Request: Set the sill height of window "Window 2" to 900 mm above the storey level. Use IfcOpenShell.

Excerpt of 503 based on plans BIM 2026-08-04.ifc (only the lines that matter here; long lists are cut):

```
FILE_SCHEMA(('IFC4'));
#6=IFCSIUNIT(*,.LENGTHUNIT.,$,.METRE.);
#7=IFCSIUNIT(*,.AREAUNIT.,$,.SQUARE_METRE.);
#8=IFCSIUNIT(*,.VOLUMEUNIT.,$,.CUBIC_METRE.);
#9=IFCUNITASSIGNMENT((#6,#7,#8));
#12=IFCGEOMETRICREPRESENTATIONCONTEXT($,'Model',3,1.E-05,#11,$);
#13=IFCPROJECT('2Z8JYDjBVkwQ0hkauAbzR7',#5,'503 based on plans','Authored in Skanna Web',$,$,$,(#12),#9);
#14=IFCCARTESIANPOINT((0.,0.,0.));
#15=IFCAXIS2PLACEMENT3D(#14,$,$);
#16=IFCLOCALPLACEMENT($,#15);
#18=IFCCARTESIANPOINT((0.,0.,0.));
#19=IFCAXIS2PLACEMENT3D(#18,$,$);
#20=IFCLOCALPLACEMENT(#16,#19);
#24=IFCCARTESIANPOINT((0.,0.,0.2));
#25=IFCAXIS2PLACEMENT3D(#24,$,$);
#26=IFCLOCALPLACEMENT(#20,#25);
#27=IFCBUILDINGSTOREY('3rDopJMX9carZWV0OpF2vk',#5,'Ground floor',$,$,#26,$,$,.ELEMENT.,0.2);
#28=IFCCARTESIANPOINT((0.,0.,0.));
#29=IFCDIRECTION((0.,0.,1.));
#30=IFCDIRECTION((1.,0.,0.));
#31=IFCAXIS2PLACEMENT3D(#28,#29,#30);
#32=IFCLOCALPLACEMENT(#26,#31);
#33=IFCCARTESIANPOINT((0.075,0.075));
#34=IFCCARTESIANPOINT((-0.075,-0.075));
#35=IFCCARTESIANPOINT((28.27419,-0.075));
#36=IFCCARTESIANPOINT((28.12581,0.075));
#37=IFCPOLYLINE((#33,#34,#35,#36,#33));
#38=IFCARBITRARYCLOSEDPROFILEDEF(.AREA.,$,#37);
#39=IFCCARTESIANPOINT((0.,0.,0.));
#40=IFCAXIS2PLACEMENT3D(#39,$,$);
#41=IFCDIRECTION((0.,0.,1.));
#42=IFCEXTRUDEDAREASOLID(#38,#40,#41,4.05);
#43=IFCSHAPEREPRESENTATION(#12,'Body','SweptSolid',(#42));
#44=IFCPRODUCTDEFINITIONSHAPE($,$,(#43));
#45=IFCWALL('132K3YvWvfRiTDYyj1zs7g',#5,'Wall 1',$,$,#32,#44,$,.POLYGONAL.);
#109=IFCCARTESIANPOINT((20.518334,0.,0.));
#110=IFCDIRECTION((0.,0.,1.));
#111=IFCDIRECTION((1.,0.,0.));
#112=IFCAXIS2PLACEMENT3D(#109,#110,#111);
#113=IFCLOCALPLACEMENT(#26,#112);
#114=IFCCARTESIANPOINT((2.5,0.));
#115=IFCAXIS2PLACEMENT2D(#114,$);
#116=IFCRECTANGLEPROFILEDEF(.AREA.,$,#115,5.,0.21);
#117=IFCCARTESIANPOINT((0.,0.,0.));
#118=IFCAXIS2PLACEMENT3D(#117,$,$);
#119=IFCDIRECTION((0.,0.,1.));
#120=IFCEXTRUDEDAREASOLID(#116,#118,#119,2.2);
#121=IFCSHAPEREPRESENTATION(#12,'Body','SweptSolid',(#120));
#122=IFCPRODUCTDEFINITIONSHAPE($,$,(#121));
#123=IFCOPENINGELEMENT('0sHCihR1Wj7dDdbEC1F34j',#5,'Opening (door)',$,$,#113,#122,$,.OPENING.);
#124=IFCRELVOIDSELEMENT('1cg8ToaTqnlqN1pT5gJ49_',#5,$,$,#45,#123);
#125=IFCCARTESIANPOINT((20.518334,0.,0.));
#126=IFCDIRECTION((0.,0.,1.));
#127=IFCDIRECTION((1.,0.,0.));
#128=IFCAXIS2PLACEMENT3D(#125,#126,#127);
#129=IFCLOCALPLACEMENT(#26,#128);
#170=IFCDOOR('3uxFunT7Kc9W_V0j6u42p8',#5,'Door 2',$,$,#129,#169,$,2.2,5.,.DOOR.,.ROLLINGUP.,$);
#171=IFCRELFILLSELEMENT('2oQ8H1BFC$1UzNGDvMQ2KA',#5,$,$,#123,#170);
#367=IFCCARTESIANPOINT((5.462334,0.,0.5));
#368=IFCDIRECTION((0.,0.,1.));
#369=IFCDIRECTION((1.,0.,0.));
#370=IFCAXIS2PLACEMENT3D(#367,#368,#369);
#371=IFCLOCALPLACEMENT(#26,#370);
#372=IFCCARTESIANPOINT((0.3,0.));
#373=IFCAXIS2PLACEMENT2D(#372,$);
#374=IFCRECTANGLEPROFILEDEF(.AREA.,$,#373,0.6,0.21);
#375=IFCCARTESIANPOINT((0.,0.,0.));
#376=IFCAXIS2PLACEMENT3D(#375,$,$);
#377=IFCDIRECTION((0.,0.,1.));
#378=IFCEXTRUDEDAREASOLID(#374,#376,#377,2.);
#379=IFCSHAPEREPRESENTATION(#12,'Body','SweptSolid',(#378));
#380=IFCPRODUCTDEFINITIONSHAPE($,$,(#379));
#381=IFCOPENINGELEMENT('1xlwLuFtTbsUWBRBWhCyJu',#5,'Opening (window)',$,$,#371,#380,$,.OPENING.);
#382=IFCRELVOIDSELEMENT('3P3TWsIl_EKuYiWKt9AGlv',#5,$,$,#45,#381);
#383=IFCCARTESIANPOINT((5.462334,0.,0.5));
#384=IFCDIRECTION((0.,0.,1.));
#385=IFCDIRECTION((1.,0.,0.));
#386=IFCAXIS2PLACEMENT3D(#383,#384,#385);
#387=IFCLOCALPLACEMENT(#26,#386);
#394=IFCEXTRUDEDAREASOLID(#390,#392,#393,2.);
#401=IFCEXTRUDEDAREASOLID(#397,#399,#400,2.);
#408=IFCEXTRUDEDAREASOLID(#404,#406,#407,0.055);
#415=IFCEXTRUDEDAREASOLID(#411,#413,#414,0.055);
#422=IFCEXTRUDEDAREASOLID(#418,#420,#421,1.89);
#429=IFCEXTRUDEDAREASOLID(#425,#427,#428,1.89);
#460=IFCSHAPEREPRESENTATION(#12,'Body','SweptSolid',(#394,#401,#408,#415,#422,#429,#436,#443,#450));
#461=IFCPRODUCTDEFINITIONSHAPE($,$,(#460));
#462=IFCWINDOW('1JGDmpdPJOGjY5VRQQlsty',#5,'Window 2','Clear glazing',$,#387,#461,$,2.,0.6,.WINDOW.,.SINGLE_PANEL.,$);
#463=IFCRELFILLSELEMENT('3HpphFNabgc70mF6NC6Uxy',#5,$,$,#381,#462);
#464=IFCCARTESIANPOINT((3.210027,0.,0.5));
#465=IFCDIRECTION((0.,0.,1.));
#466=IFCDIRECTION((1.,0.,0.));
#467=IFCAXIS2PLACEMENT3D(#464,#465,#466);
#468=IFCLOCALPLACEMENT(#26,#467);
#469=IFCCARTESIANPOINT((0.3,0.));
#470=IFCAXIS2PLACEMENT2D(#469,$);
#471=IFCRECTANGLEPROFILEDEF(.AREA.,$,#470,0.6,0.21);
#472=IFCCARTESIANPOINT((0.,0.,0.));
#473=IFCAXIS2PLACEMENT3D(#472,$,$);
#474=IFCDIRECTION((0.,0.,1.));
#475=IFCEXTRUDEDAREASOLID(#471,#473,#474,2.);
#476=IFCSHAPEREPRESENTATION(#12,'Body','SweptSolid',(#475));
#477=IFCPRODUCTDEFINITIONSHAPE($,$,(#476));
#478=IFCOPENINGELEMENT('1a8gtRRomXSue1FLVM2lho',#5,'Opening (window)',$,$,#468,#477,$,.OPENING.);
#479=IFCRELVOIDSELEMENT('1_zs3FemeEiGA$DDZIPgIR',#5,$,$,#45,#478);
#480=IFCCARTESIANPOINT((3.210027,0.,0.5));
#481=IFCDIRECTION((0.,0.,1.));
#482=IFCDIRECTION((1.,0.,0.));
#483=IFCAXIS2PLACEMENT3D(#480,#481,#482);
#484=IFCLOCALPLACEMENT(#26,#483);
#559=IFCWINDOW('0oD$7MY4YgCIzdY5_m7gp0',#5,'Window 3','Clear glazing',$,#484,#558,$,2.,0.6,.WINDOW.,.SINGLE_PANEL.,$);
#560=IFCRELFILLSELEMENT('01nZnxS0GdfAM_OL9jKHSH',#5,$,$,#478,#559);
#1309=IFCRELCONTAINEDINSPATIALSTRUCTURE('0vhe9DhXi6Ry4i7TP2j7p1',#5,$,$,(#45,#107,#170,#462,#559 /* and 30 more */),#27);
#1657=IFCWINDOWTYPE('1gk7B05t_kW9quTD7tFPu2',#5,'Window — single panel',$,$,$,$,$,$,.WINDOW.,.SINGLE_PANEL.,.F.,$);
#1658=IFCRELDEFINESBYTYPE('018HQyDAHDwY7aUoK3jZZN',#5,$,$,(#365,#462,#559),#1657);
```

```python
import numpy as np
import ifcopenshell
import ifcopenshell.api.geometry
import ifcopenshell.geom
import ifcopenshell.util.element
import ifcopenshell.util.placement
import ifcopenshell.util.shape
import ifcopenshell.util.unit

model = ifcopenshell.open("503 based on plans BIM 2026-08-04.ifc")
unit_scale = ifcopenshell.util.unit.calculate_unit_scale(model)

window = model.by_guid("1JGDmpdPJOGjY5VRQQlsty")
opening = window.FillsVoids[0].RelatingOpeningElement
storey = ifcopenshell.util.element.get_container(window, ifc_class="IfcBuildingStorey")
level = ifcopenshell.util.placement.get_local_placement(storey.ObjectPlacement)[2, 3]

# The opening's origin need not be at the sill, so measure its lowest point.
shape = ifcopenshell.geom.create_shape(ifcopenshell.geom.settings(), opening)
bottom = ifcopenshell.util.shape.get_shape_bottom_elevation(shape, shape.geometry) / unit_scale
dz = level + 0.9 - bottom

shift = np.array([0.0, 0.0, dz])
# The window is not placed relative to its opening, so move both.
for product in (opening, window):
    matrix = ifcopenshell.util.placement.get_local_placement(product.ObjectPlacement)
    matrix[:3, 3] += shift
    ifcopenshell.api.geometry.edit_object_placement(model, product=product, matrix=matrix, is_si=False)

print(f"moved by {dz * unit_scale:+.3f} m")

model.write("503 based on plans BIM 2026-08-04_v2.ifc")
```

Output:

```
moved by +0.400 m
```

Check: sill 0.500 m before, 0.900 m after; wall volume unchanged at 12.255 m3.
